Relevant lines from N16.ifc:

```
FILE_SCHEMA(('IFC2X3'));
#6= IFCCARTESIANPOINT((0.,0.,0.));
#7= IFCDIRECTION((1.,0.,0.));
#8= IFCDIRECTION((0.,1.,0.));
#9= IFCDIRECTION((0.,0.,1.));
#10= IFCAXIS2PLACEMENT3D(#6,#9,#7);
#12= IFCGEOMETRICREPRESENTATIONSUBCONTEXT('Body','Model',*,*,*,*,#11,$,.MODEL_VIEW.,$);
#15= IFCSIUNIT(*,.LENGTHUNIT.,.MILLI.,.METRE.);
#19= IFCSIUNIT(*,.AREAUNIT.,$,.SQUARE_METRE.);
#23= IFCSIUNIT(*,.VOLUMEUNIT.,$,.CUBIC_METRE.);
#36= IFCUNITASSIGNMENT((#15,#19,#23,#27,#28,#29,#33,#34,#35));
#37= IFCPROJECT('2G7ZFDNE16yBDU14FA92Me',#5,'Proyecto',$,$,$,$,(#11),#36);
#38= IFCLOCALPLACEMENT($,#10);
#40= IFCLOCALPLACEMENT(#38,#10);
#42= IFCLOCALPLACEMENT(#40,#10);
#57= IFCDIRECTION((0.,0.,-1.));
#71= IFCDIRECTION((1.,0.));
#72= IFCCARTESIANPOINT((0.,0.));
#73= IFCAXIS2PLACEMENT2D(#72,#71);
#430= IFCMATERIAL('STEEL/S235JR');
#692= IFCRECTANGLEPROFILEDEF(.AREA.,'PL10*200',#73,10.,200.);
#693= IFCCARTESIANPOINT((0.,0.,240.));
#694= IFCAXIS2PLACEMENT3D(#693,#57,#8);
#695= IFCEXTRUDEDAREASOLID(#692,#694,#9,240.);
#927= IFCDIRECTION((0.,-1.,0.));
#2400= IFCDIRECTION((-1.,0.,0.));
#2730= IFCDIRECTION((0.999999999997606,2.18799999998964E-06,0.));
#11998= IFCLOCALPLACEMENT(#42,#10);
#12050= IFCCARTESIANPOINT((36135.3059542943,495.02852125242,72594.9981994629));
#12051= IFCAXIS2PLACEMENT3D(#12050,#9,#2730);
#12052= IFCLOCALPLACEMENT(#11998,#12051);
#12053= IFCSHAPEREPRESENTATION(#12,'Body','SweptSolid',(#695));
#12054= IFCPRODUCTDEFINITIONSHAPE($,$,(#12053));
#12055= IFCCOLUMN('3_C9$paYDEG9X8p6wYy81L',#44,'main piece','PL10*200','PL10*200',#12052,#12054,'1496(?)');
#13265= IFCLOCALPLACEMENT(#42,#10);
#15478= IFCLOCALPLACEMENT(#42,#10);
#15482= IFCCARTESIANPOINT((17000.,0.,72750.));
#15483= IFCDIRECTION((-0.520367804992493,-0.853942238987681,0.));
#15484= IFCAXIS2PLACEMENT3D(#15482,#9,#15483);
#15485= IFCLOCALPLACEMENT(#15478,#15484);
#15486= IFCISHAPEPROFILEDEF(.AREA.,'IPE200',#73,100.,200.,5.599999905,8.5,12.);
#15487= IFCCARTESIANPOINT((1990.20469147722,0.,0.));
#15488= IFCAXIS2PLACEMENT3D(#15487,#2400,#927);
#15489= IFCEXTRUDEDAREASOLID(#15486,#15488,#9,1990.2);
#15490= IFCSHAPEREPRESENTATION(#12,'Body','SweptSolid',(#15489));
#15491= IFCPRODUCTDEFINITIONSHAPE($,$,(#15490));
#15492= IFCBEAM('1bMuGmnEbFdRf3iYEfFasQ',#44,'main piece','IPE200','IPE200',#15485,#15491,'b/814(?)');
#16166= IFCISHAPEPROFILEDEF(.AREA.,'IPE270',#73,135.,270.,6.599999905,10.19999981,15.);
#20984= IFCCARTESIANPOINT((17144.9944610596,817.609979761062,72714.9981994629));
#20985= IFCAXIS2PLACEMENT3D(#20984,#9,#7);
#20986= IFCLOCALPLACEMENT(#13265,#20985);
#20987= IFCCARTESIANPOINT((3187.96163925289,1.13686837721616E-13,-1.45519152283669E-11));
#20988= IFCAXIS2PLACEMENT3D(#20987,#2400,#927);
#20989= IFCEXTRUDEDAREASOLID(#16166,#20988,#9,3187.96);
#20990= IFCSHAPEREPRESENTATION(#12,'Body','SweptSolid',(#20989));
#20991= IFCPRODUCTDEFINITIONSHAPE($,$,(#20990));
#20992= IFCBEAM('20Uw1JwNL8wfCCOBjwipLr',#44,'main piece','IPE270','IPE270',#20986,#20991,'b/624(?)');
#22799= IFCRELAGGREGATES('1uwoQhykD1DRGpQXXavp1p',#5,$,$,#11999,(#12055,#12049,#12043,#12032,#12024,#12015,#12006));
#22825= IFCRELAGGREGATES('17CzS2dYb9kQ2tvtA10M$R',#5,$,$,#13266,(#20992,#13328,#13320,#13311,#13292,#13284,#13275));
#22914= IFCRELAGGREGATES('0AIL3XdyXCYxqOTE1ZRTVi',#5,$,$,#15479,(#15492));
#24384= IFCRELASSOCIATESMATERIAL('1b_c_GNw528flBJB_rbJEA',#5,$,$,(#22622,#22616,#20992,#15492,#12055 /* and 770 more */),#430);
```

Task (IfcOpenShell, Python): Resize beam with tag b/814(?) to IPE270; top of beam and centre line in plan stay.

```python
import ifcopenshell
import ifcopenshell.util.element
import ifcopenshell.util.representation

model = ifcopenshell.open("N16.ifc")

member = model.by_guid("1bMuGmnEbFdRf3iYEfFasQ")
source = next(p for p in model.by_type("IfcIShapeProfileDef") if p.ProfileName == "IPE270")

body = ifcopenshell.util.representation.get_representation(member, "Model", "Body")
solid = body.Items[0]
old_profile = solid.SweptArea

# Copy the section's sizes but keep this member's own profile position.
profile = ifcopenshell.util.element.copy(model, source)
# Profiles are centred, so shift by half the change in depth to hold the top.
shift = (old_profile.OverallDepth - profile.OverallDepth) / 2
x, y = old_profile.Position.Location.Coordinates
up = (0.0, 1.0)  # upwards, in the solid's own plane
location = model.createIfcCartesianPoint((x + up[0] * shift, y + up[1] * shift))
profile.Position = model.createIfcAxis2Placement2D(location, old_profile.Position.RefDirection)
solid.SweptArea = profile
if not model.get_total_inverses(old_profile):
    ifcopenshell.util.element.remove_deep2(model, old_profile)
member.Description = member.Description.replace("IPE200", "IPE270")
member.ObjectType = member.ObjectType.replace("IPE200", "IPE270")

print(solid.SweptArea)

model.write("N16-out.ifc")
```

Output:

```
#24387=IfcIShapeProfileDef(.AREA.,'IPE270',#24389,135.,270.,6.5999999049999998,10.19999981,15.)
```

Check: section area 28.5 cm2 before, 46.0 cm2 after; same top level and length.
